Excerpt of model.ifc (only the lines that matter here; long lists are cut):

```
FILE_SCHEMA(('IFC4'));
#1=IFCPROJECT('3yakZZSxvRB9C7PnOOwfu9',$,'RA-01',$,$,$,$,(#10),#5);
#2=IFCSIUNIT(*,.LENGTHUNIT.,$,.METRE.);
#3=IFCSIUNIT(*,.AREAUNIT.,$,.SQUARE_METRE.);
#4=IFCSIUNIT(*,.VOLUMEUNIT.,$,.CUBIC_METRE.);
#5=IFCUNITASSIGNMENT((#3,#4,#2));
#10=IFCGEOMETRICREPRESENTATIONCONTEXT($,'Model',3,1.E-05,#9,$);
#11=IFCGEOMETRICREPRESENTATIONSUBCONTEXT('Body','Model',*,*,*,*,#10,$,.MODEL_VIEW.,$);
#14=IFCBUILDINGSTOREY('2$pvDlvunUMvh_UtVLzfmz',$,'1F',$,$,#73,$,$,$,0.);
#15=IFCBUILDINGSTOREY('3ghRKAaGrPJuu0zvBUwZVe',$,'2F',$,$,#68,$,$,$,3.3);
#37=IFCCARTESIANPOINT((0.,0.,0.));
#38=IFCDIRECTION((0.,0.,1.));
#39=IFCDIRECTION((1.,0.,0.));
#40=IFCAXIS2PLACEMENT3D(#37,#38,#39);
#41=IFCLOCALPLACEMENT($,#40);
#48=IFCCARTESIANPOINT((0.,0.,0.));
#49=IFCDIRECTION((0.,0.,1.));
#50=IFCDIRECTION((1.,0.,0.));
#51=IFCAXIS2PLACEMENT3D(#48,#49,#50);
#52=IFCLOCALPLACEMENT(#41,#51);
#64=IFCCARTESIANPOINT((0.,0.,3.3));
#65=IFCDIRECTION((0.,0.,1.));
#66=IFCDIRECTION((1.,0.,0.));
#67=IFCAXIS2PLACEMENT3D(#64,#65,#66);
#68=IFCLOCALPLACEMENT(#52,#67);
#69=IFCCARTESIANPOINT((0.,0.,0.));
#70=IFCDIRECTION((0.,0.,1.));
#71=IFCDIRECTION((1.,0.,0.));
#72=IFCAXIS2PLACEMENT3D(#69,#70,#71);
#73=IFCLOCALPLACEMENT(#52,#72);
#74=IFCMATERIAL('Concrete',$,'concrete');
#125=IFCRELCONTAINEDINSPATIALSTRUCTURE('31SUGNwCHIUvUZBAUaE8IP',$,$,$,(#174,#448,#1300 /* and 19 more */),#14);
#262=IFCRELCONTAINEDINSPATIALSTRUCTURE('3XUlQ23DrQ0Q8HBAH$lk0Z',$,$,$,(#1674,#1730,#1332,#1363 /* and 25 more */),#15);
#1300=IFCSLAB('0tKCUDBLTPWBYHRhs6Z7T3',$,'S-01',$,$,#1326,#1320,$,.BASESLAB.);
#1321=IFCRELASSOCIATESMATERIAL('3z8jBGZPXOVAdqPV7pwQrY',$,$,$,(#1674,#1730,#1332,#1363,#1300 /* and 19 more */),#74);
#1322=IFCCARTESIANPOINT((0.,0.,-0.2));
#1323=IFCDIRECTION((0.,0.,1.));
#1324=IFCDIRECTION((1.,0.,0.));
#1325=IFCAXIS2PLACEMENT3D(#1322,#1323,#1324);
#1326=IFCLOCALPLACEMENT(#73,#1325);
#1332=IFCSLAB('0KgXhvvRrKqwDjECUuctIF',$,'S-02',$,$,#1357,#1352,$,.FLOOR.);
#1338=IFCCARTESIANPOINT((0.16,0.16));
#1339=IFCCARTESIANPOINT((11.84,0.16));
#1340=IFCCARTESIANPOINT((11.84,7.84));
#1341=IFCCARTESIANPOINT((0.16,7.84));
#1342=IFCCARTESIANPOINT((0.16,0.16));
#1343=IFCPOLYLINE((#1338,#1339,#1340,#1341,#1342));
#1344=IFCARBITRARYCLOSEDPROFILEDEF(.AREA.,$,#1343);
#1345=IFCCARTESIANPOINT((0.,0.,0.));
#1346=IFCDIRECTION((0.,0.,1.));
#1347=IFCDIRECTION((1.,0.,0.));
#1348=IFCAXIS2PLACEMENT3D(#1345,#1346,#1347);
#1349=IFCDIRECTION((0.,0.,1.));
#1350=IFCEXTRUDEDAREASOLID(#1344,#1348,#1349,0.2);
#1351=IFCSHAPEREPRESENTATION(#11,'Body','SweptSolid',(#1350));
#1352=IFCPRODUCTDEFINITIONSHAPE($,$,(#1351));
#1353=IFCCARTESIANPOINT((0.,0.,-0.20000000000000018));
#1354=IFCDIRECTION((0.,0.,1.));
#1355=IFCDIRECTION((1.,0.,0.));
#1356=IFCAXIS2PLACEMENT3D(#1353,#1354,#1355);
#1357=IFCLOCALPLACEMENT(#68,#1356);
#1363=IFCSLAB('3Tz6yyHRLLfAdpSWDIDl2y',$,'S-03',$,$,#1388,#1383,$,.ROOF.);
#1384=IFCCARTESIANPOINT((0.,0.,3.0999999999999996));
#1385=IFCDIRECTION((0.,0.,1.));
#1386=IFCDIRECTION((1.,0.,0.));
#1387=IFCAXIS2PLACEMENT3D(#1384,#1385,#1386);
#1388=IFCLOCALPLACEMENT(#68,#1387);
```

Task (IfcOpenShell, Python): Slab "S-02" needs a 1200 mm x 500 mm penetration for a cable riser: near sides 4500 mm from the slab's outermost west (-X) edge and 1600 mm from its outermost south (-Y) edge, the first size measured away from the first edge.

```python
import numpy as np
import ifcopenshell
import ifcopenshell.api.feature
import ifcopenshell.api.geometry
import ifcopenshell.api.root
import ifcopenshell.geom
import ifcopenshell.util.placement
import ifcopenshell.util.representation
import ifcopenshell.util.shape
import ifcopenshell.util.unit

model = ifcopenshell.open("model.ifc")
unit_scale = ifcopenshell.util.unit.calculate_unit_scale(model)
settings = ifcopenshell.geom.settings()


def volume(element):
    """Net volume in cubic metres, openings subtracted."""
    shape = ifcopenshell.geom.create_shape(settings, element)
    return ifcopenshell.util.shape.get_volume(shape.geometry)


slab = model.by_guid("0KgXhvvRrKqwDjECUuctIF")
before = volume(slab)

# Extent in the slab's own axes, in metres. The edges named are its -X and -Y sides.
slab_shape = ifcopenshell.geom.create_shape(settings, slab)
vertices = ifcopenshell.util.shape.get_vertices(slab_shape.geometry)
x_min, y_min, bottom = vertices.min(axis=0)
top = vertices[:, 2].max()

opening = ifcopenshell.api.root.create_entity(model, ifc_class="IfcOpeningElement", name="Cable riser opening", predefined_type="OPENING")
context = ifcopenshell.util.representation.get_context(model, "Model", "Body", "MODEL_VIEW")
width, depth = 1.2, 0.5
outline = [(0.0, 0.0), (width, 0.0), (width, depth), (0.0, depth), (0.0, 0.0)]
# Overshoot both faces by 50 mm so the cut is clean.
shape = ifcopenshell.api.geometry.add_slab_representation(
    model, context=context, depth=top - bottom + 0.1, polyline=outline
)
ifcopenshell.api.geometry.assign_representation(model, product=opening, representation=shape)

matrix = ifcopenshell.util.placement.get_local_placement(slab.ObjectPlacement)
matrix[:, 3] = matrix @ np.append(np.array([x_min + 4.5, y_min + 1.6, bottom - 0.05]) / unit_scale, 1.0)
ifcopenshell.api.geometry.edit_object_placement(model, product=opening, matrix=matrix, is_si=False)
ifcopenshell.api.feature.add_feature(model, feature=opening, element=slab)

after = volume(slab)

print(f"slab volume {before:.3f} -> {after:.3f} m3")

model.write("model_edited.ifc")
```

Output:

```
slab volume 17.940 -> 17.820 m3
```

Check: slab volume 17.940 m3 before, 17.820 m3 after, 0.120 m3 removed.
